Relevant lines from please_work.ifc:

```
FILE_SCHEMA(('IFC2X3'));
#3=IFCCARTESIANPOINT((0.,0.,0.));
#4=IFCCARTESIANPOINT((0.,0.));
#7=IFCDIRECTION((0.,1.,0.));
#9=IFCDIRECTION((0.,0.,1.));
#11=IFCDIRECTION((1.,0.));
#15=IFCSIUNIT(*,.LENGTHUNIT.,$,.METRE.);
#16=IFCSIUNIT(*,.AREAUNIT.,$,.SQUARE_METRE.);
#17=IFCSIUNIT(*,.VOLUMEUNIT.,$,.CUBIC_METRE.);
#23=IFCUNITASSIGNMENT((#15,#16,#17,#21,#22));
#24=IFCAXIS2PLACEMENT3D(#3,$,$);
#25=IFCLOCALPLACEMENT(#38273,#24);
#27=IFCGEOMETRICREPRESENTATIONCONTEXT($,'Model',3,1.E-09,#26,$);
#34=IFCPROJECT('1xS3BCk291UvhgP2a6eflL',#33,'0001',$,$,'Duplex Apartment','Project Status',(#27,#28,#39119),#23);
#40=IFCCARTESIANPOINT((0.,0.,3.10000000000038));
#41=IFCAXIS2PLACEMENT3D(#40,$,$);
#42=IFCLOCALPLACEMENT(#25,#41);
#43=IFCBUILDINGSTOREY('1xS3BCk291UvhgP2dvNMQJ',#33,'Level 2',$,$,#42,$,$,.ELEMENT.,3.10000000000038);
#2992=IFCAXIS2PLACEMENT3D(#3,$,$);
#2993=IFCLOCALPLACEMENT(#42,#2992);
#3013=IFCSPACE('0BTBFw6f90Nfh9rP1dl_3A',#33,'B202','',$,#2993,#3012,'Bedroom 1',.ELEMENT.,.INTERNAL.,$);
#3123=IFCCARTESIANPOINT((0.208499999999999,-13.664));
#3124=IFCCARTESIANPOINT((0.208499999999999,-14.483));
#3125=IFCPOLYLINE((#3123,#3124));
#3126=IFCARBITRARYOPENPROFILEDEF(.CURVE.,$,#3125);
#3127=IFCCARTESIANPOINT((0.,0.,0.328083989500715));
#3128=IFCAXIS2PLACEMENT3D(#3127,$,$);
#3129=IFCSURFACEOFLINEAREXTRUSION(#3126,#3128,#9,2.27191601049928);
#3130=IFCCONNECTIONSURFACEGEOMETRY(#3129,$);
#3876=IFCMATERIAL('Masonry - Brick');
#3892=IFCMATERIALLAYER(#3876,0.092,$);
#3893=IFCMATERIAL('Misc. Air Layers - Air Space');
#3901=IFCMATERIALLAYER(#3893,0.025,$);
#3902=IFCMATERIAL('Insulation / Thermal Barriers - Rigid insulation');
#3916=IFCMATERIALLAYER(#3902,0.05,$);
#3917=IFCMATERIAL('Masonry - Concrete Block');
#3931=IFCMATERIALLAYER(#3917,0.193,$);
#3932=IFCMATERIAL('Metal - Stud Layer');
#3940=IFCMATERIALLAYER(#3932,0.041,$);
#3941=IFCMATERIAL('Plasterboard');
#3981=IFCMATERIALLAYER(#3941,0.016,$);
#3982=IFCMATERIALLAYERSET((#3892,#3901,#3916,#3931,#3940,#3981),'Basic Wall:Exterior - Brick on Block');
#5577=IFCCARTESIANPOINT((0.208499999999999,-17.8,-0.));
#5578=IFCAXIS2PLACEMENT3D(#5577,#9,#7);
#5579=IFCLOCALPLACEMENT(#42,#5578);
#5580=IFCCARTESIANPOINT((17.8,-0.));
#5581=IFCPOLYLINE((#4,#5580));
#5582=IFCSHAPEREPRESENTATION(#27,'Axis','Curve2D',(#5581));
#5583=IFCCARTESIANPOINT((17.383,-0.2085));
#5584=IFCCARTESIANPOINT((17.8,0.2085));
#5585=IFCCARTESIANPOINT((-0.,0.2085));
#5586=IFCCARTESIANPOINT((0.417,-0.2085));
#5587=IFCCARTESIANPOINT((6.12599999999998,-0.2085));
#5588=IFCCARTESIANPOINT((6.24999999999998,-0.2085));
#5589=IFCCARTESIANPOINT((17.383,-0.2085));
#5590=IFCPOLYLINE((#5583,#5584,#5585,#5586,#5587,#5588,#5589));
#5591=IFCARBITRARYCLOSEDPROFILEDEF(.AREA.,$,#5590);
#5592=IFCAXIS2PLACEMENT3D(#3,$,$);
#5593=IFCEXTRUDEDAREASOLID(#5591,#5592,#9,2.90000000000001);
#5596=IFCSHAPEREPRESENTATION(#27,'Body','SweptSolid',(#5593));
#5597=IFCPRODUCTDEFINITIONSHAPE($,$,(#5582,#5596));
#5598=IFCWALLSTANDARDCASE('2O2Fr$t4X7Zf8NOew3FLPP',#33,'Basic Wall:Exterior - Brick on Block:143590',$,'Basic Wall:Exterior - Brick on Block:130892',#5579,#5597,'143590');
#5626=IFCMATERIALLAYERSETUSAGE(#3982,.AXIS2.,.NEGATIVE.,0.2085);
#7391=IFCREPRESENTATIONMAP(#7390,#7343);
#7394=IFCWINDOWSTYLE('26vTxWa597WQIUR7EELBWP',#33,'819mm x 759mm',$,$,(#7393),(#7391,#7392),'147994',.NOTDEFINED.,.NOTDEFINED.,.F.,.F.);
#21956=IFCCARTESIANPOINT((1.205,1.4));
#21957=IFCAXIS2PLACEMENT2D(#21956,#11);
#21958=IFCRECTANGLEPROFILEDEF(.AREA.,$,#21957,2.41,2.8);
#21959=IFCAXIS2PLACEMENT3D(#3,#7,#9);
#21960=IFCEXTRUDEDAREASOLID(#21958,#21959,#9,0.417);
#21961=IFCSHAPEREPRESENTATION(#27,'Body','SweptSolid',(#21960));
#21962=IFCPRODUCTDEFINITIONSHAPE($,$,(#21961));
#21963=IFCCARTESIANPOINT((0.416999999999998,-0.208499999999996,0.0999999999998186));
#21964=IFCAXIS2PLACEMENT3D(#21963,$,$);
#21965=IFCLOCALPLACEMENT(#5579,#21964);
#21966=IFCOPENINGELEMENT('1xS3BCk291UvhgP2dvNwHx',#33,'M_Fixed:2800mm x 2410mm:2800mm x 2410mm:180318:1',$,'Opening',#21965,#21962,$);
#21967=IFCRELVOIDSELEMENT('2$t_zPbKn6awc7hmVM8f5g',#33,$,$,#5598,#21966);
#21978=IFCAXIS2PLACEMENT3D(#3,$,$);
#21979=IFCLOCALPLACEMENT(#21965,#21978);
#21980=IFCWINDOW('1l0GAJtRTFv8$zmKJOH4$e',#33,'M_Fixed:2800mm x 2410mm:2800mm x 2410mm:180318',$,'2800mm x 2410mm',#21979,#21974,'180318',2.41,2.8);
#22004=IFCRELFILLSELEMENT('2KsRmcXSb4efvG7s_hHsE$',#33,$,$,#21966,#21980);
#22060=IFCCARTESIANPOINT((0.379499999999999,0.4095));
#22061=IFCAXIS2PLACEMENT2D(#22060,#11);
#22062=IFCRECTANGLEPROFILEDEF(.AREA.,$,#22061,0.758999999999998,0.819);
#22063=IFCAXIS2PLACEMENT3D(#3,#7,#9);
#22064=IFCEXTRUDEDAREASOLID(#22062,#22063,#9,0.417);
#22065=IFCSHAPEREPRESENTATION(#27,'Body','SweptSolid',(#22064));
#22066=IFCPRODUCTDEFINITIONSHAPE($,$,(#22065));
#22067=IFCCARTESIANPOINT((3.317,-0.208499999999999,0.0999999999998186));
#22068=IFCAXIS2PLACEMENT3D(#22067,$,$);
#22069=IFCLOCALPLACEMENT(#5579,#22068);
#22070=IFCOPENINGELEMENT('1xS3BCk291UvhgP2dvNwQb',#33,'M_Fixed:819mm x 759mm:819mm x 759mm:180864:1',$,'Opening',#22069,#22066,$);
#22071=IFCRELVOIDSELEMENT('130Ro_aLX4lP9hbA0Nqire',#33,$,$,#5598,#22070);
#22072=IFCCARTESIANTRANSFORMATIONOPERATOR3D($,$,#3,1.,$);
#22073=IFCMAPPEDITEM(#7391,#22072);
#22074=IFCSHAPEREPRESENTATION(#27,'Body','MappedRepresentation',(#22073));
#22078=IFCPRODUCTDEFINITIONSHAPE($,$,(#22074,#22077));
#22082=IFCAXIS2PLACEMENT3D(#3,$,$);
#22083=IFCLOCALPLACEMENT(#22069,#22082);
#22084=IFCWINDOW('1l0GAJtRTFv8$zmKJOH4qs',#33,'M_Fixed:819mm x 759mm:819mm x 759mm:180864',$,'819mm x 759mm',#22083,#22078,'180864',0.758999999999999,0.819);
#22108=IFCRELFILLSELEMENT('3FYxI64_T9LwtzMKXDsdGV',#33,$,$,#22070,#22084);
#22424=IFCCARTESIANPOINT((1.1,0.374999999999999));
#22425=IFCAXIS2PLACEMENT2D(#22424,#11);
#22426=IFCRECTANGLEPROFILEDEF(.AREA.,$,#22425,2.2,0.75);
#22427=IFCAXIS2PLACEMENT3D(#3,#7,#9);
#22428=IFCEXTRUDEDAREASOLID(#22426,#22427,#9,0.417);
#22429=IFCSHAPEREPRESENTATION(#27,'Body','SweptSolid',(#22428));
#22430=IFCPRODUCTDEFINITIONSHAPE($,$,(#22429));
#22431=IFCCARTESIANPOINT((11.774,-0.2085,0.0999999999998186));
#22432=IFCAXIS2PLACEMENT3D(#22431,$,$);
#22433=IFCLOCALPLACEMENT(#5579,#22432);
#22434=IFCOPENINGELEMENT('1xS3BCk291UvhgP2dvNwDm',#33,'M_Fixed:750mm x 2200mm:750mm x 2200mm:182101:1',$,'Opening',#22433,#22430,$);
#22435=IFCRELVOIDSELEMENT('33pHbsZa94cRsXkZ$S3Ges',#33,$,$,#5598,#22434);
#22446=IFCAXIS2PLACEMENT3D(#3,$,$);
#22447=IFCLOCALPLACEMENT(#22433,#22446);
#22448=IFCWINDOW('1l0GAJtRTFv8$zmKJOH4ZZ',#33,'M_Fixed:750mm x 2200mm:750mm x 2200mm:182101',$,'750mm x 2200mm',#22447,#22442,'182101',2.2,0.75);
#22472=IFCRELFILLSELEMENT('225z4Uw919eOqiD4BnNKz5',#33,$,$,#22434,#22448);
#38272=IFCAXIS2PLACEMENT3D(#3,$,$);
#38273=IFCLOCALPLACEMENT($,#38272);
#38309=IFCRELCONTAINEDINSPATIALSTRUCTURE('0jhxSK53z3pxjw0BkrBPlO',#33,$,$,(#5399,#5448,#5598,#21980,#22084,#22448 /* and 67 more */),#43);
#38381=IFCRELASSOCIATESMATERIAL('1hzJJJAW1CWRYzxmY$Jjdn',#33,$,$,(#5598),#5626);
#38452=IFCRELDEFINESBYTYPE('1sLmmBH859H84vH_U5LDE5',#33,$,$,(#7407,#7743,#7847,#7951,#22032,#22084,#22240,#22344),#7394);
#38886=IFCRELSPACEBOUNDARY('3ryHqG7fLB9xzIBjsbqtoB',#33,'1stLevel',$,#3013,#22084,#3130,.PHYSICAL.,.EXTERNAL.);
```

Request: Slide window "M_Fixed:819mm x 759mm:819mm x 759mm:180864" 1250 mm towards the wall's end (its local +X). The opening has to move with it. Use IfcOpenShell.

```python
import numpy as np
import ifcopenshell
import ifcopenshell.api.geometry
import ifcopenshell.util.placement
import ifcopenshell.util.unit

model = ifcopenshell.open("please_work.ifc")
unit_scale = ifcopenshell.util.unit.calculate_unit_scale(model)

window = model.by_id(22084)
opening = window.FillsVoids[0].RelatingOpeningElement
wall = opening.VoidsElements[0].RelatingBuildingElement

wall_matrix = ifcopenshell.util.placement.get_local_placement(wall.ObjectPlacement)
shift = wall_matrix[:3, 0] * 1.25 / unit_scale
before = ifcopenshell.util.placement.get_local_placement(window.ObjectPlacement)[:3, 3].copy()

# The window is placed relative to its opening, so it follows when the opening moves.
matrix = ifcopenshell.util.placement.get_local_placement(opening.ObjectPlacement)
matrix[:3, 3] += shift
ifcopenshell.api.geometry.edit_object_placement(
    model, product=opening, matrix=matrix, is_si=False, should_transform_children=True
)

# Space boundary surfaces are stored in each space's coordinates; move them too.
for rel in window.ProvidesBoundaries:
    if not rel.ConnectionGeometry:
        continue
    surface = rel.ConnectionGeometry.SurfaceOnRelatingElement
    space_matrix = ifcopenshell.util.placement.get_local_placement(rel.RelatingSpace.ObjectPlacement)
    point = np.array(surface.Position.Location.Coordinates) + space_matrix[:3, :3].T @ shift
    surface.Position = model.createIfcAxis2Placement3D(
        model.createIfcCartesianPoint(point.tolist()), surface.Position.Axis, surface.Position.RefDirection
    )

after = ifcopenshell.util.placement.get_local_placement(window.ObjectPlacement)[:3, 3]
print("window moved by", (after - before).round(3) + 0.0)

model.write("please_work_edited.ifc")
```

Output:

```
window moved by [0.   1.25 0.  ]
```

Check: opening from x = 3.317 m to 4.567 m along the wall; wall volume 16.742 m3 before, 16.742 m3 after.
